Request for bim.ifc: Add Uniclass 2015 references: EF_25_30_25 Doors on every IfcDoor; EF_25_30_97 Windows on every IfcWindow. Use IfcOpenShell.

First a look at what the model holds.

```python
import ifcopenshell

model = ifcopenshell.open("bim.ifc")
print(model.schema)
print("classifications:", [c.Name for c in model.by_type("IfcClassification")])
for ifc_class in ("IfcDoor", "IfcRoof", "IfcStair", "IfcWall", "IfcWindow"):
    print(ifc_class, len(model.by_type(ifc_class)))
```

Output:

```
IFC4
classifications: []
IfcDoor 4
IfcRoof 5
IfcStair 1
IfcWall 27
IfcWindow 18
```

```python
import ifcopenshell
import ifcopenshell.api.classification

model = ifcopenshell.open("bim.ifc")

system = ifcopenshell.api.classification.add_classification(model, classification="Uniclass 2015")

codes = {
    "IfcDoor": ("EF_25_30_25", "Doors"),
    "IfcWindow": ("EF_25_30_97", "Windows"),
}
for ifc_class, (code, name) in codes.items():
    products = model.by_type(ifc_class)
    ifcopenshell.api.classification.add_reference(
        model, products=products, classification=system, identification=code, name=name
    )
    print(code, len(products))

model.write("bim_edited.ifc")
```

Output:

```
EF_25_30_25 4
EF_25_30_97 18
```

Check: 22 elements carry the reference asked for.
